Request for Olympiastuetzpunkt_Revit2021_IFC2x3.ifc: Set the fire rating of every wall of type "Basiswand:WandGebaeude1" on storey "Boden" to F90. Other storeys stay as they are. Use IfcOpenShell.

First a look at what the model holds.

```python
import ifcopenshell
import ifcopenshell.util.element

model = ifcopenshell.open("Olympiastuetzpunkt_Revit2021_IFC2x3.ifc")
print(model.schema)
storey = next(s for s in model.by_type("IfcBuildingStorey") if s.Name == "Boden")
walls = [e for e in ifcopenshell.util.element.get_decomposition(storey) if e.is_a("IfcWall")]
seen = {}
for e in walls:
    element_type = ifcopenshell.util.element.get_type(e)
    key = (element_type.Name if element_type != e and element_type else None, ifcopenshell.util.element.get_pset(e, "Pset_WallCommon", "FireRating"))
    seen[key] = seen.get(key, 0) + 1
for (name, value), count in sorted(seen.items(), key=str):
    print(count, "x", name, "|", value)
```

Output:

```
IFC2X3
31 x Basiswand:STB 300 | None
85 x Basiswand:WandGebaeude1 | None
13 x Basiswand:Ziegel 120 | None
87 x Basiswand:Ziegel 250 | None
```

```python
import ifcopenshell
import ifcopenshell.api.pset
import ifcopenshell.util.element

model = ifcopenshell.open("Olympiastuetzpunkt_Revit2021_IFC2x3.ifc")

storey = next(s for s in model.by_type("IfcBuildingStorey") if s.Name == "Boden")
walls = [e for e in ifcopenshell.util.element.get_decomposition(storey) if e.is_a("IfcWall")]

count = 0
for e in walls:
    element_type = ifcopenshell.util.element.get_type(e)
    if element_type in (None, e) or element_type.Name != "Basiswand:WandGebaeude1":
        continue
    # add_pset returns the element's existing set when there is one.
    pset = ifcopenshell.api.pset.add_pset(model, product=e, name="Pset_WallCommon")
    ifcopenshell.api.pset.edit_pset(model, pset=pset, properties={"FireRating": "F90"})
    count += 1

print(count, "walls updated")

model.write("Olympiastuetzpunkt_Revit2021_IFC2x3-out.ifc")
```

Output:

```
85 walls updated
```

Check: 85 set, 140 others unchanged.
